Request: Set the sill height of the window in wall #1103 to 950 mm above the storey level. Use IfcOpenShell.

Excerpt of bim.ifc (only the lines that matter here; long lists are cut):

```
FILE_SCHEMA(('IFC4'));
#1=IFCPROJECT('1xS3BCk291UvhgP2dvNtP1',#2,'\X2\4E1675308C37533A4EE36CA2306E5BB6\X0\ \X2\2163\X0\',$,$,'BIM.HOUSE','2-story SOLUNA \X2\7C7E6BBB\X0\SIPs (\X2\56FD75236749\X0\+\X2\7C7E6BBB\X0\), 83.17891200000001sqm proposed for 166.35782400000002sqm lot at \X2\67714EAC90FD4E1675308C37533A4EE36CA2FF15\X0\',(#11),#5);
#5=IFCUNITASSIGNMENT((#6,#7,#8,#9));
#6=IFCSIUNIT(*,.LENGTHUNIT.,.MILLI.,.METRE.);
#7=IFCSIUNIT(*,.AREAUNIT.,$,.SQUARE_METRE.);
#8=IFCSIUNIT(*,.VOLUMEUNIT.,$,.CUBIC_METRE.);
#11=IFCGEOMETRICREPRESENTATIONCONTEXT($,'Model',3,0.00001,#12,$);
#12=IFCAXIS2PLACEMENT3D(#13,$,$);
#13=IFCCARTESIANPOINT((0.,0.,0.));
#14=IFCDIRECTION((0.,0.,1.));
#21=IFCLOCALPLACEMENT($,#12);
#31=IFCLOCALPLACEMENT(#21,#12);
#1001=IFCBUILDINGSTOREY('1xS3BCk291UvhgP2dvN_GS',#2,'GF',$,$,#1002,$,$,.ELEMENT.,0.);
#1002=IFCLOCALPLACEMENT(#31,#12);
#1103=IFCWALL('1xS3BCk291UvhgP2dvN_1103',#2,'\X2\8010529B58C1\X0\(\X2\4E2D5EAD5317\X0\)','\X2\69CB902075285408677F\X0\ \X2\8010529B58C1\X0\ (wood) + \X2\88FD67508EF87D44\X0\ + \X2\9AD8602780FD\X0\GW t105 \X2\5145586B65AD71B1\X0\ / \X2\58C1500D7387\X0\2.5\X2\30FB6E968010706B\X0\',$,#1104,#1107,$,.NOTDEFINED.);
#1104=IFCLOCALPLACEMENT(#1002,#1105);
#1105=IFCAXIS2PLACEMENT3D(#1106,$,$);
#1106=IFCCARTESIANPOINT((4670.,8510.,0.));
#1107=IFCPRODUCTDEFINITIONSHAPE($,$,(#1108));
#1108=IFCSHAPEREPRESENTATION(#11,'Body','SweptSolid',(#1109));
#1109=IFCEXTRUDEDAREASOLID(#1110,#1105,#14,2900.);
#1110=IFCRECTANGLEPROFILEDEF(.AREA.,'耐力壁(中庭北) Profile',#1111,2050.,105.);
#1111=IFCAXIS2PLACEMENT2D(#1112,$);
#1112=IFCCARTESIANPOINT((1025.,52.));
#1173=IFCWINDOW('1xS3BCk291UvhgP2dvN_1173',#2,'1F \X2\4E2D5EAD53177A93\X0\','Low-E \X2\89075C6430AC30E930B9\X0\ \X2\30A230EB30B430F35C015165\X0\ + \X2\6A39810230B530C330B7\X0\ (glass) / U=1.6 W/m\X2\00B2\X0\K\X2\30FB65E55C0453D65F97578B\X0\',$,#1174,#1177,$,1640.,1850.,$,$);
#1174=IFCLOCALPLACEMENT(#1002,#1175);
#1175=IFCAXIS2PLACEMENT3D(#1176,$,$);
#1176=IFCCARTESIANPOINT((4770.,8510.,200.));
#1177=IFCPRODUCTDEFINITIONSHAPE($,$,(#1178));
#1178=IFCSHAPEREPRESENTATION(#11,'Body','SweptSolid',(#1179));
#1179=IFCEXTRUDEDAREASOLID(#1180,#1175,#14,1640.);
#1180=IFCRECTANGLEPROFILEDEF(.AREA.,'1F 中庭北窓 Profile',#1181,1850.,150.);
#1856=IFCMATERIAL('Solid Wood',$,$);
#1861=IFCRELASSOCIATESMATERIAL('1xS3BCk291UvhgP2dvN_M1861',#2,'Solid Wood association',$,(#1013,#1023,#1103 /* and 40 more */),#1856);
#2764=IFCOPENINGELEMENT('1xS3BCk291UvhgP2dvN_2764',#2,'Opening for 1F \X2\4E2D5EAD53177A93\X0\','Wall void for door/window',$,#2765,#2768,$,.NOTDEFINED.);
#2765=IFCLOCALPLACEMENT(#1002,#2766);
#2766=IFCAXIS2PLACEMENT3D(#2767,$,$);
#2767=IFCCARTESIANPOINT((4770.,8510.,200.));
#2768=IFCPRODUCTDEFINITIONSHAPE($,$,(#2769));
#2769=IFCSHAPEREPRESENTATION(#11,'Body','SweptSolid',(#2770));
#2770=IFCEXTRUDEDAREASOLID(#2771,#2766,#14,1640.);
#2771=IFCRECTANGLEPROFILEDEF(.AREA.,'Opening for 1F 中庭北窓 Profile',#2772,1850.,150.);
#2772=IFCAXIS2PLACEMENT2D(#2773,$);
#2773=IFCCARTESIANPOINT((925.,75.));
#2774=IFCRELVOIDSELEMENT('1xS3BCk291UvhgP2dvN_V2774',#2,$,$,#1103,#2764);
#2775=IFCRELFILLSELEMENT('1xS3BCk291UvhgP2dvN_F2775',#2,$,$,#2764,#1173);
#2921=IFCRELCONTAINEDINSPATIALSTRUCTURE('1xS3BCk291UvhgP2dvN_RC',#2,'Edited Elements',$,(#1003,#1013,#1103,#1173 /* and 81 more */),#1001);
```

```python
import numpy as np
import ifcopenshell
import ifcopenshell.api.geometry
import ifcopenshell.geom
import ifcopenshell.util.element
import ifcopenshell.util.placement
import ifcopenshell.util.shape
import ifcopenshell.util.unit

model = ifcopenshell.open("bim.ifc")
unit_scale = ifcopenshell.util.unit.calculate_unit_scale(model)

window = model.by_guid("1xS3BCk291UvhgP2dvN_1173")
opening = window.FillsVoids[0].RelatingOpeningElement
storey = ifcopenshell.util.element.get_container(window, ifc_class="IfcBuildingStorey")
level = ifcopenshell.util.placement.get_local_placement(storey.ObjectPlacement)[2, 3]

# The opening's origin need not be at the sill, so measure its lowest point.
shape = ifcopenshell.geom.create_shape(ifcopenshell.geom.settings(), opening)
bottom = ifcopenshell.util.shape.get_shape_bottom_elevation(shape, shape.geometry) / unit_scale
dz = level + 0.95 / unit_scale - bottom

shift = np.array([0.0, 0.0, dz])
# The window is not placed relative to its opening, so move both.
for product in (opening, window):
    matrix = ifcopenshell.util.placement.get_local_placement(product.ObjectPlacement)
    matrix[:3, 3] += shift
    ifcopenshell.api.geometry.edit_object_placement(model, product=product, matrix=matrix, is_si=False)

print(f"moved by {dz * unit_scale:+.3f} m")

model.write("bim_rev.ifc")
```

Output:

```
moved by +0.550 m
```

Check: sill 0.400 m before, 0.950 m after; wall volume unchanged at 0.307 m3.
